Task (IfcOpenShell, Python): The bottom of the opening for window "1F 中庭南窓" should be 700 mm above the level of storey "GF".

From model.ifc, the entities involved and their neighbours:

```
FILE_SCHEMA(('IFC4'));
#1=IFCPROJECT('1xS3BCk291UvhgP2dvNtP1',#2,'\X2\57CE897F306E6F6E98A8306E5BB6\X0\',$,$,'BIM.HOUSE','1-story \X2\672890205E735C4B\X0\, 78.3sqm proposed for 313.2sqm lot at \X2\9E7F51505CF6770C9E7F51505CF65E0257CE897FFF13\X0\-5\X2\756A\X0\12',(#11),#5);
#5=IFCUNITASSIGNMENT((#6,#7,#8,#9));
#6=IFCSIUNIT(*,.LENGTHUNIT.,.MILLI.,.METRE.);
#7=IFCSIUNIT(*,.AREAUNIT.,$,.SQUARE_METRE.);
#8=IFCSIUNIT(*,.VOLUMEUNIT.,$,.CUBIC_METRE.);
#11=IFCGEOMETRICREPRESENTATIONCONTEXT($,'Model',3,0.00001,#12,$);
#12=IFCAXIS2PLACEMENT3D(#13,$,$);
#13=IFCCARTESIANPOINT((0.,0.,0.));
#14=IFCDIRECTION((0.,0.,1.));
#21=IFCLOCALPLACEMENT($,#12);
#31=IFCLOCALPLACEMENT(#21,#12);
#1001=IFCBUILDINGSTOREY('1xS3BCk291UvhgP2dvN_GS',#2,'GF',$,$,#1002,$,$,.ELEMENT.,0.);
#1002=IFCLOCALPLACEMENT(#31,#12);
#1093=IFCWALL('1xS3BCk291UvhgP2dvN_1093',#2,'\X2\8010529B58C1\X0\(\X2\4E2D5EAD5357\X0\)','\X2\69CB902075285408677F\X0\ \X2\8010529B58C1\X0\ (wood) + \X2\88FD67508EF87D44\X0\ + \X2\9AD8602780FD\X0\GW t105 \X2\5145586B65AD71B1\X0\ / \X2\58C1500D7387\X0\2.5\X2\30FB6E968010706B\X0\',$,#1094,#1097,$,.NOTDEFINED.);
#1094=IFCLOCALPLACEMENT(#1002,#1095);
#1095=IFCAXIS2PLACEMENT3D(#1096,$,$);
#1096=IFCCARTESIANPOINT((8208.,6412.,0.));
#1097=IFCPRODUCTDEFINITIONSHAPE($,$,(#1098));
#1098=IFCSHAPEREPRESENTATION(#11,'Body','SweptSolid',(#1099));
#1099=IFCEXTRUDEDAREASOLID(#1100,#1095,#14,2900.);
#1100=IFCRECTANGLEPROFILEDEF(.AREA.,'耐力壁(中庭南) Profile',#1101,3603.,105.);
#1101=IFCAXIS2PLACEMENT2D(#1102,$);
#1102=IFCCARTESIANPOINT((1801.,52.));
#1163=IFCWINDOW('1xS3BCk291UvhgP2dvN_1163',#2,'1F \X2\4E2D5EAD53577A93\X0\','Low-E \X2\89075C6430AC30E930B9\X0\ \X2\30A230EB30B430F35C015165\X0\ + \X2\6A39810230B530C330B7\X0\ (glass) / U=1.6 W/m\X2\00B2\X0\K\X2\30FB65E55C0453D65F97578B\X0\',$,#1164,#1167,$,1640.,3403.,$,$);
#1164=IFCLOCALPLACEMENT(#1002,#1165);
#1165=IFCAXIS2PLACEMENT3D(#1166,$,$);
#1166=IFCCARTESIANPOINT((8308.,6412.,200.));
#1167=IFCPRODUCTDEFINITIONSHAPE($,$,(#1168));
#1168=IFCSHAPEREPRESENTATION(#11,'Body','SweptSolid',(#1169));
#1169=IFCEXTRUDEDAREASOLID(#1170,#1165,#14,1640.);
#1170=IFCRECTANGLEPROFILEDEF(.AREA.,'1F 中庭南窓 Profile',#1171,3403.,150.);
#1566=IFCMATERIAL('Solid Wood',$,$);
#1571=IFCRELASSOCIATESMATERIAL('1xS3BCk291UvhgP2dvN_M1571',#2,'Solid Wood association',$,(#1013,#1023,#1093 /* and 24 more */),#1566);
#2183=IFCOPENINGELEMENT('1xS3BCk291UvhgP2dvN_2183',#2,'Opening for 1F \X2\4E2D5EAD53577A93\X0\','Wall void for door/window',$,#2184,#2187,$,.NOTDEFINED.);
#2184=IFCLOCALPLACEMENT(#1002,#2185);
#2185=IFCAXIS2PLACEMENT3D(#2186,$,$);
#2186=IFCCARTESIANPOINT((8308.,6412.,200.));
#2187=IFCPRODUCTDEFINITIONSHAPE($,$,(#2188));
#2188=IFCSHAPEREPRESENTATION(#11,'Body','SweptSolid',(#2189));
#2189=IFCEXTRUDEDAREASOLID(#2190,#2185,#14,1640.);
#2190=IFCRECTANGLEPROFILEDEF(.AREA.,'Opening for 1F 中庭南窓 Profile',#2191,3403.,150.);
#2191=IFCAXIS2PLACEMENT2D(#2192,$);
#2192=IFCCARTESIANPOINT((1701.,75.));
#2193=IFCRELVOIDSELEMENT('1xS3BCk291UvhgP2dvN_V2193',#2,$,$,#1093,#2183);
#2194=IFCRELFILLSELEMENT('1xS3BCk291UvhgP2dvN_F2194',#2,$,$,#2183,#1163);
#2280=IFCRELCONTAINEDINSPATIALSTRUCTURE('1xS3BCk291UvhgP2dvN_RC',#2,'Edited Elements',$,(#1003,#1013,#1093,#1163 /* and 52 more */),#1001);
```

```python
import numpy as np
import ifcopenshell
import ifcopenshell.api.geometry
import ifcopenshell.geom
import ifcopenshell.util.element
import ifcopenshell.util.placement
import ifcopenshell.util.shape
import ifcopenshell.util.unit

model = ifcopenshell.open("model.ifc")
unit_scale = ifcopenshell.util.unit.calculate_unit_scale(model)

window = model.by_guid("1xS3BCk291UvhgP2dvN_1163")
opening = window.FillsVoids[0].RelatingOpeningElement
storey = ifcopenshell.util.element.get_container(window, ifc_class="IfcBuildingStorey")
level = ifcopenshell.util.placement.get_local_placement(storey.ObjectPlacement)[2, 3]

# The opening's origin need not be at the sill, so measure its lowest point.
shape = ifcopenshell.geom.create_shape(ifcopenshell.geom.settings(), opening)
bottom = ifcopenshell.util.shape.get_shape_bottom_elevation(shape, shape.geometry) / unit_scale
dz = level + 700.0 - bottom

shift = np.array([0.0, 0.0, dz])
# The window is not placed relative to its opening, so move both.
for product in (opening, window):
    matrix = ifcopenshell.util.placement.get_local_placement(product.ObjectPlacement)
    matrix[:3, 3] += shift
    ifcopenshell.api.geometry.edit_object_placement(model, product=product, matrix=matrix, is_si=False)

print(f"moved by {dz * unit_scale:+.3f} m")

model.write("model_v2.ifc")
```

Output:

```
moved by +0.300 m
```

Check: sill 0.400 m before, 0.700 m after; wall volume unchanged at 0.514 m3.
